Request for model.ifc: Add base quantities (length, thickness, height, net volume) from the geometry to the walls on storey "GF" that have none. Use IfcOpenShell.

First a look at what the model holds.

```python
import ifcopenshell
import ifcopenshell.util.element
import ifcopenshell.util.unit

model = ifcopenshell.open("model.ifc")
print(model.schema)
for unit_type in ("LENGTHUNIT", "AREAUNIT", "VOLUMEUNIT"):
    print(unit_type, ifcopenshell.util.unit.calculate_unit_scale(model, unit_type))
storey = next(s for s in model.by_type("IfcBuildingStorey") if s.Name == "GF")
walls = [e for e in ifcopenshell.util.element.get_decomposition(storey) if e.is_a("IfcWall")]
for e in sorted(walls, key=lambda e: e.id()):
    print(e.id(), e.is_a(), e.Name, list(ifcopenshell.util.element.get_psets(e, qtos_only=True)), sep=" | ")
```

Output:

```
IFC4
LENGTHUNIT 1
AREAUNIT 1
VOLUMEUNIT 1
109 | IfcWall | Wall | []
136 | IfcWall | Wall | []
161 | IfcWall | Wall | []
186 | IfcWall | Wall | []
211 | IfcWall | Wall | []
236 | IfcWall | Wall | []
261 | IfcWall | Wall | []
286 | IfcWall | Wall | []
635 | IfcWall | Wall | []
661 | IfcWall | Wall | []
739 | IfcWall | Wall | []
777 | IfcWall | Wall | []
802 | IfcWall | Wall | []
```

```python
import ifcopenshell
import ifcopenshell.api.pset
import ifcopenshell.geom
import ifcopenshell.util.element
import ifcopenshell.util.shape
import ifcopenshell.util.unit

model = ifcopenshell.open("model.ifc")
unit_scale = ifcopenshell.util.unit.calculate_unit_scale(model)
volume_scale = ifcopenshell.util.unit.calculate_unit_scale(model, "VOLUMEUNIT")
settings = ifcopenshell.geom.settings()

storey = next(s for s in model.by_type("IfcBuildingStorey") if s.Name == "GF")
walls = [e for e in ifcopenshell.util.element.get_decomposition(storey) if e.is_a("IfcWall")]

for e in sorted(walls, key=lambda e: e.id()):
    if ifcopenshell.util.element.get_psets(e, qtos_only=True, should_inherit=False):
        continue
    # Geometry comes back in metres, in the element's own axes.
    shape = ifcopenshell.geom.create_shape(settings, e)
    values = {
        "Length": ifcopenshell.util.shape.get_x(shape.geometry) / unit_scale,
        "Width": ifcopenshell.util.shape.get_y(shape.geometry) / unit_scale,
        "Height": ifcopenshell.util.shape.get_z(shape.geometry) / unit_scale,
        "NetVolume": ifcopenshell.util.shape.get_volume(shape.geometry) / volume_scale,
    }
    qto = ifcopenshell.api.pset.add_qto(model, product=e, name="Qto_WallBaseQuantities")
    ifcopenshell.api.pset.edit_qto(model, qto=qto, properties=values)
    print(e.id(), {k: round(v, 3) for k, v in values.items()})

model.write("model-out.ifc")
```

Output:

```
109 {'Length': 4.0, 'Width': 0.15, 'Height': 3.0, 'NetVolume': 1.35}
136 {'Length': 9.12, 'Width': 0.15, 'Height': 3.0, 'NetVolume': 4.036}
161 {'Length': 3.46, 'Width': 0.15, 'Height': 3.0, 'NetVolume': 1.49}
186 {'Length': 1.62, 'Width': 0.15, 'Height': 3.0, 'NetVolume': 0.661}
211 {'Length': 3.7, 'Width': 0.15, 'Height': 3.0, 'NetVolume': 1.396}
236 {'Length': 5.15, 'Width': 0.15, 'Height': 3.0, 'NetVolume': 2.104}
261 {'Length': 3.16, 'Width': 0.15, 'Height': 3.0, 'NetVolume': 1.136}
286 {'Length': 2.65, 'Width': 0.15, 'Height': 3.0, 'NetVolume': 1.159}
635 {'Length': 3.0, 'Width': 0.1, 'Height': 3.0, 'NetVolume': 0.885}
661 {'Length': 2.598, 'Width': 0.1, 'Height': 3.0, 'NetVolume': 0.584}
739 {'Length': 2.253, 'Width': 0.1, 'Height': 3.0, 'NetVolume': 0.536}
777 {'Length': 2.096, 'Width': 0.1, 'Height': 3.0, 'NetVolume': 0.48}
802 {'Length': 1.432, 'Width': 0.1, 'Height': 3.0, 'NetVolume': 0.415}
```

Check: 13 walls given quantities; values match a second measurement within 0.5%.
